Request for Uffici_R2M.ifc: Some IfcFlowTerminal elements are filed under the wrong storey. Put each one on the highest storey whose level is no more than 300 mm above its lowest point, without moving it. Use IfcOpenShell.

First a look at what the model holds.

```python
import ifcopenshell
import ifcopenshell.util.element
import ifcopenshell.util.placement

model = ifcopenshell.open("Uffici_R2M.ifc")
print(model.schema)
for storey in model.by_type("IfcBuildingStorey"):
    level = ifcopenshell.util.placement.get_storey_elevation(storey)
    count = sum(e.is_a("IfcFlowTerminal") for e in ifcopenshell.util.element.get_contained(storey))
    print(storey.id(), storey.Name, round(level, 3), count, sep=" | ")
```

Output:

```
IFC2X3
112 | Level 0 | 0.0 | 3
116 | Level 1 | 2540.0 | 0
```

```python
import ifcopenshell
import ifcopenshell.api.spatial
import ifcopenshell.geom
import ifcopenshell.util.element
import ifcopenshell.util.placement
import ifcopenshell.util.shape
import ifcopenshell.util.unit

model = ifcopenshell.open("Uffici_R2M.ifc")
unit_scale = ifcopenshell.util.unit.calculate_unit_scale(model)
settings = ifcopenshell.geom.settings()

levels = sorted(
    ((ifcopenshell.util.placement.get_storey_elevation(s) * unit_scale, s) for s in model.by_type("IfcBuildingStorey")),
    key=lambda pair: pair[0],
)

for e in model.by_type("IfcFlowTerminal"):
    current = e.ContainedInStructure[0].RelatingStructure if e.ContainedInStructure else None
    if current is None or not current.is_a("IfcBuildingStorey"):
        continue
    shape = ifcopenshell.geom.create_shape(settings, e)
    bottom = ifcopenshell.util.shape.get_shape_bottom_elevation(shape, shape.geometry)
    below = [s for level, s in levels if level <= bottom + 0.3]
    storey = below[-1] if below else levels[0][1]
    if storey != current:
        # assign_container keeps the world position.
        ifcopenshell.api.spatial.assign_container(model, products=[e], relating_structure=storey)
        print(e.id(), current.Name, "->", storey.Name)

model.write("Uffici_R2M_edited.ifc")
```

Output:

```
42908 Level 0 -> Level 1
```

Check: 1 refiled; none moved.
